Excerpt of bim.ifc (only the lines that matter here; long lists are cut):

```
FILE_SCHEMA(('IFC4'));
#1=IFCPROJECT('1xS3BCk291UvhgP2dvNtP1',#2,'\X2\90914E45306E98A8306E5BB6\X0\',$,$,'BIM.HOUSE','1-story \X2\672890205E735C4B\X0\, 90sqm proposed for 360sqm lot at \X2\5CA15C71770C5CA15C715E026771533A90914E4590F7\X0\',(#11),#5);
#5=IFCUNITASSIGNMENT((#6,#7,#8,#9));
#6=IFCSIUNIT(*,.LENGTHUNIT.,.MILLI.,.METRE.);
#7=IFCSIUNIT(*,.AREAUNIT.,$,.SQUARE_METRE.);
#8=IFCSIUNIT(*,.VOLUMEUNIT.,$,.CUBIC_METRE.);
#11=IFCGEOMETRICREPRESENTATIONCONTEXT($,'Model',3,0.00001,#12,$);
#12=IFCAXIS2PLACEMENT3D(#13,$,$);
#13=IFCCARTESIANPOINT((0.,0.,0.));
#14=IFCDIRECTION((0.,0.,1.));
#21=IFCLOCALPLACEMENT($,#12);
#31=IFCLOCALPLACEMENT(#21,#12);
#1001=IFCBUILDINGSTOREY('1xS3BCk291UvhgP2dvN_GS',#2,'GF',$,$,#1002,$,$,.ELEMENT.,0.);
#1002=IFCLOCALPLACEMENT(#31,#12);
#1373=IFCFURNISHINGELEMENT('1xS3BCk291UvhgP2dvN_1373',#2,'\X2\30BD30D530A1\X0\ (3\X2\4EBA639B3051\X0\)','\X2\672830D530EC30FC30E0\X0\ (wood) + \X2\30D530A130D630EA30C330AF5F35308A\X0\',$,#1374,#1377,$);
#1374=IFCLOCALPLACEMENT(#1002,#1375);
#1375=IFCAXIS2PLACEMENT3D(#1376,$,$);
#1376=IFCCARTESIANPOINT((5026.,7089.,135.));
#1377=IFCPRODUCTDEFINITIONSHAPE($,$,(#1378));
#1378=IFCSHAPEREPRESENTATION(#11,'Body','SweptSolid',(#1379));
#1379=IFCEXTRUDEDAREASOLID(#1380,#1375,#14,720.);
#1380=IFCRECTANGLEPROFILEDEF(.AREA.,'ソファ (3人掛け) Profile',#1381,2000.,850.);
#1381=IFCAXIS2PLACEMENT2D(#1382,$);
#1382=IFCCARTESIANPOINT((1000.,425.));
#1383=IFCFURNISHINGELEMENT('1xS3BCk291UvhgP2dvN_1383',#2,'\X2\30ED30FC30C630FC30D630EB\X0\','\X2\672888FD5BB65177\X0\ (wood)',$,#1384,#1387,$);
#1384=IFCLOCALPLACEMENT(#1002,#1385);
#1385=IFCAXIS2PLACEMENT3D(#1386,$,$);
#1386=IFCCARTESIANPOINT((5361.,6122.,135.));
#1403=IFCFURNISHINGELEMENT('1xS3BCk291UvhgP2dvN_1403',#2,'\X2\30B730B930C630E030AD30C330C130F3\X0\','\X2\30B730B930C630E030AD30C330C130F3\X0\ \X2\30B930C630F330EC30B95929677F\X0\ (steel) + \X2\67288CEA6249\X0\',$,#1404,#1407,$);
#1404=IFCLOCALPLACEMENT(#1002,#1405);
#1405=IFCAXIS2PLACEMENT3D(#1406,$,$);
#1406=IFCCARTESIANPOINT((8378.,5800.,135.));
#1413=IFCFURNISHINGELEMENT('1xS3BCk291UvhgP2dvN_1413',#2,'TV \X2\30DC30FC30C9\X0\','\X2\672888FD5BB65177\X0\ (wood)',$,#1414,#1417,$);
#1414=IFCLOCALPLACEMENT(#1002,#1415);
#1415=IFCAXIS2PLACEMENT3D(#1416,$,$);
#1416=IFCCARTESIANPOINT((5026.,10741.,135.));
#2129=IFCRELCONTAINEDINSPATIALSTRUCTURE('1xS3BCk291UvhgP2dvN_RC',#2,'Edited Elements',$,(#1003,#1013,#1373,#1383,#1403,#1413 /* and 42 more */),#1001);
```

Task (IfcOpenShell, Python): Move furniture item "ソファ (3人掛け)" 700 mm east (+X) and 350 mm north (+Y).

```python
import ifcopenshell
import ifcopenshell.api.geometry
import ifcopenshell.util.placement
import ifcopenshell.util.unit

model = ifcopenshell.open("bim.ifc")
unit_scale = ifcopenshell.util.unit.calculate_unit_scale(model)

item = model.by_guid("1xS3BCk291UvhgP2dvN_1373")
matrix = ifcopenshell.util.placement.get_local_placement(item.ObjectPlacement)
matrix[0, 3] += 0.7 / unit_scale
matrix[1, 3] += 0.35 / unit_scale
ifcopenshell.api.geometry.edit_object_placement(model, product=item, matrix=matrix, is_si=False)

print(ifcopenshell.util.placement.get_local_placement(item.ObjectPlacement).round(3) + 0.0)

model.write("bim_rev.ifc")
```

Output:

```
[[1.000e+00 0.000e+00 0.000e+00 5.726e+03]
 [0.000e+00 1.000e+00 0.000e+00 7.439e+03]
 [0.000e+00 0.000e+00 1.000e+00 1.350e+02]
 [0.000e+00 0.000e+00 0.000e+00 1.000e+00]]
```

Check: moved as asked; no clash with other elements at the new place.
